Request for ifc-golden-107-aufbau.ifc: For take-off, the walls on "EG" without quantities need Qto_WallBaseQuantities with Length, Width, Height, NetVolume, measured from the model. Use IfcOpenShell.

First a look at what the model holds.

```python
import ifcopenshell
import ifcopenshell.util.element
import ifcopenshell.util.unit

model = ifcopenshell.open("ifc-golden-107-aufbau.ifc")
print(model.schema)
for unit_type in ("LENGTHUNIT", "AREAUNIT", "VOLUMEUNIT"):
    print(unit_type, ifcopenshell.util.unit.calculate_unit_scale(model, unit_type))
storey = next(s for s in model.by_type("IfcBuildingStorey") if s.Name == "EG")
walls = [e for e in ifcopenshell.util.element.get_decomposition(storey) if e.is_a("IfcWall")]
for e in sorted(walls, key=lambda e: e.id()):
    print(e.id(), e.is_a(), e.Name, list(ifcopenshell.util.element.get_psets(e, qtos_only=True)), sep=" | ")
```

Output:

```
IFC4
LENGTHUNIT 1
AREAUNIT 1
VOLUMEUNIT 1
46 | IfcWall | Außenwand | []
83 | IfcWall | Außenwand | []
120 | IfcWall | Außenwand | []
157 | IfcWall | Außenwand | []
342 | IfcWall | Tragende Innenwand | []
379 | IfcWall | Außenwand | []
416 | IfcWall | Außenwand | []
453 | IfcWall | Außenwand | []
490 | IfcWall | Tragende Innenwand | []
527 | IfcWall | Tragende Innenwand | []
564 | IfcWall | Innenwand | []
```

```python
import ifcopenshell
import ifcopenshell.api.pset
import ifcopenshell.geom
import ifcopenshell.util.element
import ifcopenshell.util.shape
import ifcopenshell.util.unit

model = ifcopenshell.open("ifc-golden-107-aufbau.ifc")
unit_scale = ifcopenshell.util.unit.calculate_unit_scale(model)
volume_scale = ifcopenshell.util.unit.calculate_unit_scale(model, "VOLUMEUNIT")
settings = ifcopenshell.geom.settings()

storey = next(s for s in model.by_type("IfcBuildingStorey") if s.Name == "EG")
walls = [e for e in ifcopenshell.util.element.get_decomposition(storey) if e.is_a("IfcWall")]

for e in sorted(walls, key=lambda e: e.id()):
    if ifcopenshell.util.element.get_psets(e, qtos_only=True, should_inherit=False):
        continue
    # Geometry comes back in metres, in the element's own axes.
    shape = ifcopenshell.geom.create_shape(settings, e)
    values = {
        "Length": ifcopenshell.util.shape.get_x(shape.geometry) / unit_scale,
        "Width": ifcopenshell.util.shape.get_y(shape.geometry) / unit_scale,
        "Height": ifcopenshell.util.shape.get_z(shape.geometry) / unit_scale,
        "NetVolume": ifcopenshell.util.shape.get_volume(shape.geometry) / volume_scale,
    }
    qto = ifcopenshell.api.pset.add_qto(model, product=e, name="Qto_WallBaseQuantities")
    ifcopenshell.api.pset.edit_qto(model, qto=qto, properties=values)
    print(e.id(), {k: round(v, 3) for k, v in values.items()})

model.write("ifc-golden-107-aufbau_updated.ifc")
```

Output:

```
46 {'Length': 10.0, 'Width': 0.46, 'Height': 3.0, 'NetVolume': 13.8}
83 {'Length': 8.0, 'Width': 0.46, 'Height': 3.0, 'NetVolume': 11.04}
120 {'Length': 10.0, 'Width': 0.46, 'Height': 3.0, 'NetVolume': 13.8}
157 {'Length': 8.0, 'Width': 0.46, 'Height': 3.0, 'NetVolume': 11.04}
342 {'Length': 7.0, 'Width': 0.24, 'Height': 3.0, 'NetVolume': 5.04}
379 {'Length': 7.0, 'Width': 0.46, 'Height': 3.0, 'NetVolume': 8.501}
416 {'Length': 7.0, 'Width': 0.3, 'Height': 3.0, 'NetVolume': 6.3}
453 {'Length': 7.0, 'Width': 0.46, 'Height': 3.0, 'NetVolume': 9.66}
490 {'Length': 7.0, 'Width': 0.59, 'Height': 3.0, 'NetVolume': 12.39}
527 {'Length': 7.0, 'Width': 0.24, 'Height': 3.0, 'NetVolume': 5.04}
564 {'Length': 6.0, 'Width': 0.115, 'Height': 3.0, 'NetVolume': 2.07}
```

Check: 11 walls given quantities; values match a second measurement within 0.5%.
